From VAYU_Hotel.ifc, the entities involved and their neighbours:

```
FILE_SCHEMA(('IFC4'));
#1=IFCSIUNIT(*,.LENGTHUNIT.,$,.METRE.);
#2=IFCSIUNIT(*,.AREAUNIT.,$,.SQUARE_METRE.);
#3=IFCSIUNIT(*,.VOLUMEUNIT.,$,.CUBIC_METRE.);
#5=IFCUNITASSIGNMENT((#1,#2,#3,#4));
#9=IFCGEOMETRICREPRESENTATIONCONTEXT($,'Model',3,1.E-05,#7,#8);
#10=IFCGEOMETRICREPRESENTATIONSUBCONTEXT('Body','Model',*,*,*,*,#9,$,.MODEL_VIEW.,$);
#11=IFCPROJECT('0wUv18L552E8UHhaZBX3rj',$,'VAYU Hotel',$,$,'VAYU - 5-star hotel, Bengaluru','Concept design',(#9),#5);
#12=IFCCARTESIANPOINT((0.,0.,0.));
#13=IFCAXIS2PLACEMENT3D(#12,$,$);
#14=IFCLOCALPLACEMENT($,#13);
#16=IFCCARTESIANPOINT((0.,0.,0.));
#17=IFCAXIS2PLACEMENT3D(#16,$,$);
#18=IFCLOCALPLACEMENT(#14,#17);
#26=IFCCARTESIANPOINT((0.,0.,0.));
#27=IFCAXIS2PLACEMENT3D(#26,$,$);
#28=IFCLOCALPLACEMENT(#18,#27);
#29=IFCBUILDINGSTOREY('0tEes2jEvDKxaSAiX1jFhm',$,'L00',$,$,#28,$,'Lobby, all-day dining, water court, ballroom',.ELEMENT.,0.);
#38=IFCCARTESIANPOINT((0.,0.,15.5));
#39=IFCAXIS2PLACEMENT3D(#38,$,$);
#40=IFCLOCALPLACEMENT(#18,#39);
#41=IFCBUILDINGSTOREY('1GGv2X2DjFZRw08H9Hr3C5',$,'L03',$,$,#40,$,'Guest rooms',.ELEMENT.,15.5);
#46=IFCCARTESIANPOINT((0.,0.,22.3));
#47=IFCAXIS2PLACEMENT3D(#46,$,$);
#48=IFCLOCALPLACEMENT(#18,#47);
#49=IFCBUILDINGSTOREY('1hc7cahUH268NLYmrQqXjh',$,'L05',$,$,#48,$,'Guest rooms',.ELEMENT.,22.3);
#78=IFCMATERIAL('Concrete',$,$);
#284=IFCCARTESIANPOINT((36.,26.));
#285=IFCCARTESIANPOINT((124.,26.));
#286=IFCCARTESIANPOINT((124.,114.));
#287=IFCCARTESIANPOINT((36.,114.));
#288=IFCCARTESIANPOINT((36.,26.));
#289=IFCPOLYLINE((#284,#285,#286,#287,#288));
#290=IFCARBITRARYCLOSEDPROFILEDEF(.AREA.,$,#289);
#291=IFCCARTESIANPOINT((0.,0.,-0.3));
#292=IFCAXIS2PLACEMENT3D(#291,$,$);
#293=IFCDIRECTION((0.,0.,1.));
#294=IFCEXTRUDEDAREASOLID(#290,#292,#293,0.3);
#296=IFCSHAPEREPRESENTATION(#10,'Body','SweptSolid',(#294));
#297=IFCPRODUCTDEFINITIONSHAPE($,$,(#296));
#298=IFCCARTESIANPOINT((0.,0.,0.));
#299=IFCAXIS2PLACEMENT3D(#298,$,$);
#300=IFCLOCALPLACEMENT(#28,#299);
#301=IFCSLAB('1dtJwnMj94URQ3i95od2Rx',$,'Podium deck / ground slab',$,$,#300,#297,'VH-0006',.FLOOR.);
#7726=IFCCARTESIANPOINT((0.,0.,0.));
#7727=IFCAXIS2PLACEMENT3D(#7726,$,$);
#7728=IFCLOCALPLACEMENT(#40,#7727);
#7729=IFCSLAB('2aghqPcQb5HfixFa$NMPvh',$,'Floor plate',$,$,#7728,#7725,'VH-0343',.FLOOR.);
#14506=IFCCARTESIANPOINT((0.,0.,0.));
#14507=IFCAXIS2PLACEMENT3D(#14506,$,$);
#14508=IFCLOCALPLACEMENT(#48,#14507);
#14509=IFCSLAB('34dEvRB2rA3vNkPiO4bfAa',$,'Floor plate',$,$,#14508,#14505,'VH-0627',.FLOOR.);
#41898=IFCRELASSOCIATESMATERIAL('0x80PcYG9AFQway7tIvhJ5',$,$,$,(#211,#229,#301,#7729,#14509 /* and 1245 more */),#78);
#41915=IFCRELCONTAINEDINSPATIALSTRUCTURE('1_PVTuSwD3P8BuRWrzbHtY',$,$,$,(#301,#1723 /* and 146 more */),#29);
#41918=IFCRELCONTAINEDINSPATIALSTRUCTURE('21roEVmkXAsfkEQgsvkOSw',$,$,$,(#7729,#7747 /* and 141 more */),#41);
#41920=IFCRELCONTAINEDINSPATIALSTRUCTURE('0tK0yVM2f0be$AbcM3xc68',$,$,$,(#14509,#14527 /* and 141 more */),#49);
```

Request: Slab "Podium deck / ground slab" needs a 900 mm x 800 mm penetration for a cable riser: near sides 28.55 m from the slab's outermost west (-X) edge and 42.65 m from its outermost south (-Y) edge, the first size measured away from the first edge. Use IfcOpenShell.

```python
import numpy as np
import ifcopenshell
import ifcopenshell.api.feature
import ifcopenshell.api.geometry
import ifcopenshell.api.root
import ifcopenshell.geom
import ifcopenshell.util.placement
import ifcopenshell.util.representation
import ifcopenshell.util.shape
import ifcopenshell.util.unit

model = ifcopenshell.open("VAYU_Hotel.ifc")
unit_scale = ifcopenshell.util.unit.calculate_unit_scale(model)
settings = ifcopenshell.geom.settings()


def volume(element):
    """Net volume in cubic metres, openings subtracted."""
    shape = ifcopenshell.geom.create_shape(settings, element)
    return ifcopenshell.util.shape.get_volume(shape.geometry)


slab = model.by_guid("1dtJwnMj94URQ3i95od2Rx")
before = volume(slab)

# Extent in the slab's own axes, in metres. The edges named are its -X and -Y sides.
slab_shape = ifcopenshell.geom.create_shape(settings, slab)
vertices = ifcopenshell.util.shape.get_vertices(slab_shape.geometry)
x_min, y_min, bottom = vertices.min(axis=0)
top = vertices[:, 2].max()

opening = ifcopenshell.api.root.create_entity(model, ifc_class="IfcOpeningElement", name="Cable riser opening", predefined_type="OPENING")
context = ifcopenshell.util.representation.get_context(model, "Model", "Body", "MODEL_VIEW")
width, depth = 0.9, 0.8
outline = [(0.0, 0.0), (width, 0.0), (width, depth), (0.0, depth), (0.0, 0.0)]
# Overshoot both faces by 50 mm so the cut is clean.
shape = ifcopenshell.api.geometry.add_slab_representation(
    model, context=context, depth=top - bottom + 0.1, polyline=outline
)
ifcopenshell.api.geometry.assign_representation(model, product=opening, representation=shape)

matrix = ifcopenshell.util.placement.get_local_placement(slab.ObjectPlacement)
matrix[:, 3] = matrix @ np.append(np.array([x_min + 28.55, y_min + 42.65, bottom - 0.05]) / unit_scale, 1.0)
ifcopenshell.api.geometry.edit_object_placement(model, product=opening, matrix=matrix, is_si=False)
ifcopenshell.api.feature.add_feature(model, feature=opening, element=slab)

after = volume(slab)

print(f"slab volume {before:.3f} -> {after:.3f} m3")

model.write("VAYU_Hotel_rev.ifc")
```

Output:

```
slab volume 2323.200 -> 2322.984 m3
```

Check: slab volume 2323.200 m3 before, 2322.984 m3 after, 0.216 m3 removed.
